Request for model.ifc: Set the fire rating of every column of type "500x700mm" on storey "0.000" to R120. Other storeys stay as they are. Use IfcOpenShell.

First a look at what the model holds.

```python
import ifcopenshell
import ifcopenshell.util.element

model = ifcopenshell.open("model.ifc")
print(model.schema)
storey = next(s for s in model.by_type("IfcBuildingStorey") if s.Name == "0.000")
columns = [e for e in ifcopenshell.util.element.get_decomposition(storey) if e.is_a("IfcColumn")]
seen = {}
for e in columns:
    element_type = ifcopenshell.util.element.get_type(e)
    key = (element_type.Name if element_type != e and element_type else None, ifcopenshell.util.element.get_pset(e, "Pset_ColumnCommon", "FireRating"))
    seen[key] = seen.get(key, 0) + 1
for (name, value), count in sorted(seen.items(), key=str):
    print(count, "x", name, "|", value)
```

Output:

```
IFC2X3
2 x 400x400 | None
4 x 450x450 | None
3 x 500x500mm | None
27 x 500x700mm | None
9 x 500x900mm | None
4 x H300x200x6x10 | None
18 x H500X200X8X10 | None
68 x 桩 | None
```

```python
import ifcopenshell
import ifcopenshell.api.pset
import ifcopenshell.util.element

model = ifcopenshell.open("model.ifc")

storey = next(s for s in model.by_type("IfcBuildingStorey") if s.Name == "0.000")
columns = [e for e in ifcopenshell.util.element.get_decomposition(storey) if e.is_a("IfcColumn")]

count = 0
for e in columns:
    element_type = ifcopenshell.util.element.get_type(e)
    if element_type in (None, e) or element_type.Name != "500x700mm":
        continue
    # add_pset returns the element's existing set when there is one.
    pset = ifcopenshell.api.pset.add_pset(model, product=e, name="Pset_ColumnCommon")
    ifcopenshell.api.pset.edit_pset(model, pset=pset, properties={"FireRating": "R120"})
    count += 1

print(count, "columns updated")

model.write("model_updated.ifc")
```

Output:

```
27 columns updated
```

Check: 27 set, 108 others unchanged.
